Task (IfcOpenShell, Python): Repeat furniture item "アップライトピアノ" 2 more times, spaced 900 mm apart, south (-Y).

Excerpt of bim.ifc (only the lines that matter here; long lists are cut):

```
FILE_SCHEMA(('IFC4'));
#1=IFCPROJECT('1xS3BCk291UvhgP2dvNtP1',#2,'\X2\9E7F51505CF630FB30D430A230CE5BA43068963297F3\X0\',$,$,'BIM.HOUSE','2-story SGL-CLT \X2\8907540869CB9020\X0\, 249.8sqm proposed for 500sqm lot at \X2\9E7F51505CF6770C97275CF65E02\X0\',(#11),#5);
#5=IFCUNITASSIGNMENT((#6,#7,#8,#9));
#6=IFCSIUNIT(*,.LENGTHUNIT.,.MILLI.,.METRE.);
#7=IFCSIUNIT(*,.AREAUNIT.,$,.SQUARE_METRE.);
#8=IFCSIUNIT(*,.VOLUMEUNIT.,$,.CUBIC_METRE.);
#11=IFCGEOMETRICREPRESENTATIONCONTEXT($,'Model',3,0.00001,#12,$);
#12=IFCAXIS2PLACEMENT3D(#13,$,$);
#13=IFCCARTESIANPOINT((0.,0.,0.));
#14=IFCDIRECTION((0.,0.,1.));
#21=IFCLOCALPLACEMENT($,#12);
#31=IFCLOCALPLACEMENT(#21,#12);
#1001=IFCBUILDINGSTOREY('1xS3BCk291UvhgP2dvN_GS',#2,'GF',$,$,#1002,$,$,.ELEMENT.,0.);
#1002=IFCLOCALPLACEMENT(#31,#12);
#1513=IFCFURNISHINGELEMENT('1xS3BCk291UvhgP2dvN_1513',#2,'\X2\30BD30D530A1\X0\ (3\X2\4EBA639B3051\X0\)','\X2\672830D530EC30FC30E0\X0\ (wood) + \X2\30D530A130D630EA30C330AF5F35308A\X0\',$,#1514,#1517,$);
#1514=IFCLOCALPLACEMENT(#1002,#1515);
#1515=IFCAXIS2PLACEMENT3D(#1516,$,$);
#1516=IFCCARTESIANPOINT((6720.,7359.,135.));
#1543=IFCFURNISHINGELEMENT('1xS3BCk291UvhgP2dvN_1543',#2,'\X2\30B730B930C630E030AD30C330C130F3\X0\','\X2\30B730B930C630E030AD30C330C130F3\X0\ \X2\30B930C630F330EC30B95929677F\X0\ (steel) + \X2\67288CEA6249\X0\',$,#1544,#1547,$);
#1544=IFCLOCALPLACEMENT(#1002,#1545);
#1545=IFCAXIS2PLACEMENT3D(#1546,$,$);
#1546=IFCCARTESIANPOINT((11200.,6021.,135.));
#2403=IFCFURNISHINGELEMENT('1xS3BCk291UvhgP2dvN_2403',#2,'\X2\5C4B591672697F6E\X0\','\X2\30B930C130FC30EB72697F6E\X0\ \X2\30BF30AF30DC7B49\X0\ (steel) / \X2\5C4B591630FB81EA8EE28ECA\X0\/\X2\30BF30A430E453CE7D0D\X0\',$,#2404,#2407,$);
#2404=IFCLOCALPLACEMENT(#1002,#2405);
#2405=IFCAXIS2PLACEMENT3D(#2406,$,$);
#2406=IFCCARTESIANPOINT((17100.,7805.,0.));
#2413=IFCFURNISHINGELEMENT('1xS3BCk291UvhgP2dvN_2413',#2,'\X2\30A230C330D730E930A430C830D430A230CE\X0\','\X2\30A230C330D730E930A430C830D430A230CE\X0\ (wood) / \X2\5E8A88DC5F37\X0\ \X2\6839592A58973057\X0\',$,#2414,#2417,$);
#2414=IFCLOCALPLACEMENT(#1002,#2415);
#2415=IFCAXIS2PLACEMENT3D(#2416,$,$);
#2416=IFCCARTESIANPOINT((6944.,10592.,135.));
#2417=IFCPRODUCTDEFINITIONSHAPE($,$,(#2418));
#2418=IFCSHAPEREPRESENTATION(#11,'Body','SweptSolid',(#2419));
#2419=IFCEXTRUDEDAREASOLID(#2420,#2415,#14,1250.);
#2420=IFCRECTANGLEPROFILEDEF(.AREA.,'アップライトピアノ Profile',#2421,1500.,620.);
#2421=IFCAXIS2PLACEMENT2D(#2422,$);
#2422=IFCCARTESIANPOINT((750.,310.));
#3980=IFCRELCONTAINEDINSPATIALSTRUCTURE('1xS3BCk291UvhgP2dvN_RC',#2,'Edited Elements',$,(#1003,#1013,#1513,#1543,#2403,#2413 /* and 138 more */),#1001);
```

```python
import numpy as np
import ifcopenshell
import ifcopenshell.api.geometry
import ifcopenshell.api.root
import ifcopenshell.util.element
import ifcopenshell.util.placement

model = ifcopenshell.open("bim.ifc")


def reuse_history(source, copy):
    """copy_class also copies each property set's owner history, people and application; keep the originals."""
    for rel in copy.IsDefinedBy:
        if rel.is_a("IfcRelDefinesByProperties") and (history := rel.RelatingPropertyDefinition.OwnerHistory):
            rel.RelatingPropertyDefinition.OwnerHistory = source.OwnerHistory
            ifcopenshell.util.element.remove_deep2(model, history)


source = model.by_guid("1xS3BCk291UvhgP2dvN_2413")
base = ifcopenshell.util.placement.get_local_placement(source.ObjectPlacement)
step = np.array([0.0, -1.0, 0.0]) * 900.0

for i in range(1, 3):
    copy = ifcopenshell.api.root.copy_class(model, product=source)
    copy.Representation = ifcopenshell.util.element.copy_deep(
        model, source.Representation, exclude=["IfcGeometricRepresentationContext", "IfcRepresentationMap"]
    )
    reuse_history(source, copy)
    matrix = base.copy()
    matrix[:3, 3] += i * step
    print("added at", matrix[:3, 3].round(3) + 0.0)
    ifcopenshell.api.geometry.edit_object_placement(model, product=copy, matrix=matrix, is_si=False)

model.write("bim_v2.ifc")
```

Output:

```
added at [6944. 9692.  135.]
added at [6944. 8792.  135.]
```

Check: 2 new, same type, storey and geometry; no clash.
